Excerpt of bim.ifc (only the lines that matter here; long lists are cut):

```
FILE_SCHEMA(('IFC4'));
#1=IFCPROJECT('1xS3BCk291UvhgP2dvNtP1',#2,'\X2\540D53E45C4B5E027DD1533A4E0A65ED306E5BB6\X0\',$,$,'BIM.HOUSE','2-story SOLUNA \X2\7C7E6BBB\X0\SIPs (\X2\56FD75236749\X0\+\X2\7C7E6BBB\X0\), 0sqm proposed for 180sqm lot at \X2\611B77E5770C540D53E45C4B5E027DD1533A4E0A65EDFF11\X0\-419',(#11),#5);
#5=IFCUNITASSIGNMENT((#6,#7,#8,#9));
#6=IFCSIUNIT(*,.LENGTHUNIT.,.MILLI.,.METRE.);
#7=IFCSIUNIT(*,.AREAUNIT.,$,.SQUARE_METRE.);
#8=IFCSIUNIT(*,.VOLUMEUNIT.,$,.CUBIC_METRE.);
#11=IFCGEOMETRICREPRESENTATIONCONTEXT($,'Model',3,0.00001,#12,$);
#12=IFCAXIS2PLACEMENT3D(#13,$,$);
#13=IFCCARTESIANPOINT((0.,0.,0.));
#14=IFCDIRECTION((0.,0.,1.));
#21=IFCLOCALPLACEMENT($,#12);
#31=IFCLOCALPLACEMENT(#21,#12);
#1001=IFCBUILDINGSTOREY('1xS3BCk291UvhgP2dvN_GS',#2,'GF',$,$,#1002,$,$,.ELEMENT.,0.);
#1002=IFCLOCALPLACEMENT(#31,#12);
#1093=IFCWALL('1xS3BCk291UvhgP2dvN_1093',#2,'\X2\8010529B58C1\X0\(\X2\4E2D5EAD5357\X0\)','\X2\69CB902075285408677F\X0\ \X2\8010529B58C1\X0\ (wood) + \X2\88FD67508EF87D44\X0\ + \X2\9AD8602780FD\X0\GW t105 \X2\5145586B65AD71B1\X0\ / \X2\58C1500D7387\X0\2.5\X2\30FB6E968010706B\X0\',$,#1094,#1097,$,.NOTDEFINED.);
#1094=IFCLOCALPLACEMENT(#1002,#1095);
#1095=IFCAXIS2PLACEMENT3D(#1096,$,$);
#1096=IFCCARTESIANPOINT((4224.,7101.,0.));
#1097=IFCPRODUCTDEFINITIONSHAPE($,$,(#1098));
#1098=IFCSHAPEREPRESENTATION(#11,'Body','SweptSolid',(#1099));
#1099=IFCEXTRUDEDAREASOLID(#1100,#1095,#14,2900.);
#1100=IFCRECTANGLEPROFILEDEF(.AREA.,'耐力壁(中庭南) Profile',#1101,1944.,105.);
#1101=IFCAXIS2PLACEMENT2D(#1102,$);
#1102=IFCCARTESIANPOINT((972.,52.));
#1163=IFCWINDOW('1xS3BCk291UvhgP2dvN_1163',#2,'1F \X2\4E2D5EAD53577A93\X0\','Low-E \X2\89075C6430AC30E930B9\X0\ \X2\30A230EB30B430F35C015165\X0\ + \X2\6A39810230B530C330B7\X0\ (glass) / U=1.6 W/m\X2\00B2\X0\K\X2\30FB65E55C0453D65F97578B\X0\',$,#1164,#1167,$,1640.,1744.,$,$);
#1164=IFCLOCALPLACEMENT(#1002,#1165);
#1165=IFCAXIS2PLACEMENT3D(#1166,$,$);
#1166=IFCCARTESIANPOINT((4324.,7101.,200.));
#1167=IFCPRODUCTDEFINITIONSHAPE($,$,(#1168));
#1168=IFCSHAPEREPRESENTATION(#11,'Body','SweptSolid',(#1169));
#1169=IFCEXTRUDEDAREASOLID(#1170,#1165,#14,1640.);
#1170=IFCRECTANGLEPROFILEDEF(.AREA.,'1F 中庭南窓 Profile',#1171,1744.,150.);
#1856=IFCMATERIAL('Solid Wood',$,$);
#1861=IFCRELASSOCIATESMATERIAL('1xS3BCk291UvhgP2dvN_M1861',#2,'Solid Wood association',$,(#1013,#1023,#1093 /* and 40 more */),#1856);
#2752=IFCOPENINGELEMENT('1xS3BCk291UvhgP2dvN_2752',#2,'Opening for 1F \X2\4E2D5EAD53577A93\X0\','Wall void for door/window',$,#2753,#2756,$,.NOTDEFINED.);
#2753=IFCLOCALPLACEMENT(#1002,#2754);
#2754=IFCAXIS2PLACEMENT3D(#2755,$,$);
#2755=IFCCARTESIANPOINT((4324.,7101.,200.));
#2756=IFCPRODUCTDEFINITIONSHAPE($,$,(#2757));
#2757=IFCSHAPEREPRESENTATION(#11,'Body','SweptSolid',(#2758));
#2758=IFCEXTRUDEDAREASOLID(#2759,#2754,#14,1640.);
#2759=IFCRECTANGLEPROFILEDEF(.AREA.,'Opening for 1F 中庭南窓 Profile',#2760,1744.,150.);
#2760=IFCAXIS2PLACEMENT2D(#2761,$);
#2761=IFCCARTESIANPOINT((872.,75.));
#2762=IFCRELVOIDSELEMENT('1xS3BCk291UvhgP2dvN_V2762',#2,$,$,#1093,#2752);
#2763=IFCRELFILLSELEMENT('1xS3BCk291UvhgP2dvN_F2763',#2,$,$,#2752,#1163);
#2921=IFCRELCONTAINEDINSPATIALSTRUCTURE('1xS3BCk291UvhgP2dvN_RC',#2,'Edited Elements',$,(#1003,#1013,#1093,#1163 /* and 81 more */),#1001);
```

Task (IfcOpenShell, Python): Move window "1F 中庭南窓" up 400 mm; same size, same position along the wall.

```python
import numpy as np
import ifcopenshell
import ifcopenshell.api.geometry
import ifcopenshell.util.placement
import ifcopenshell.util.unit

model = ifcopenshell.open("bim.ifc")
unit_scale = ifcopenshell.util.unit.calculate_unit_scale(model)

window = model.by_guid("1xS3BCk291UvhgP2dvN_1163")
opening = window.FillsVoids[0].RelatingOpeningElement
dz = 0.4 / unit_scale

shift = np.array([0.0, 0.0, dz])
# The window is not placed relative to its opening, so move both.
for product in (opening, window):
    matrix = ifcopenshell.util.placement.get_local_placement(product.ObjectPlacement)
    matrix[:3, 3] += shift
    ifcopenshell.api.geometry.edit_object_placement(model, product=product, matrix=matrix, is_si=False)

print(f"moved by {dz * unit_scale:+.3f} m")

model.write("bim-out.ifc")
```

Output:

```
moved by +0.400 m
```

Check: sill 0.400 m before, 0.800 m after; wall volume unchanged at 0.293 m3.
